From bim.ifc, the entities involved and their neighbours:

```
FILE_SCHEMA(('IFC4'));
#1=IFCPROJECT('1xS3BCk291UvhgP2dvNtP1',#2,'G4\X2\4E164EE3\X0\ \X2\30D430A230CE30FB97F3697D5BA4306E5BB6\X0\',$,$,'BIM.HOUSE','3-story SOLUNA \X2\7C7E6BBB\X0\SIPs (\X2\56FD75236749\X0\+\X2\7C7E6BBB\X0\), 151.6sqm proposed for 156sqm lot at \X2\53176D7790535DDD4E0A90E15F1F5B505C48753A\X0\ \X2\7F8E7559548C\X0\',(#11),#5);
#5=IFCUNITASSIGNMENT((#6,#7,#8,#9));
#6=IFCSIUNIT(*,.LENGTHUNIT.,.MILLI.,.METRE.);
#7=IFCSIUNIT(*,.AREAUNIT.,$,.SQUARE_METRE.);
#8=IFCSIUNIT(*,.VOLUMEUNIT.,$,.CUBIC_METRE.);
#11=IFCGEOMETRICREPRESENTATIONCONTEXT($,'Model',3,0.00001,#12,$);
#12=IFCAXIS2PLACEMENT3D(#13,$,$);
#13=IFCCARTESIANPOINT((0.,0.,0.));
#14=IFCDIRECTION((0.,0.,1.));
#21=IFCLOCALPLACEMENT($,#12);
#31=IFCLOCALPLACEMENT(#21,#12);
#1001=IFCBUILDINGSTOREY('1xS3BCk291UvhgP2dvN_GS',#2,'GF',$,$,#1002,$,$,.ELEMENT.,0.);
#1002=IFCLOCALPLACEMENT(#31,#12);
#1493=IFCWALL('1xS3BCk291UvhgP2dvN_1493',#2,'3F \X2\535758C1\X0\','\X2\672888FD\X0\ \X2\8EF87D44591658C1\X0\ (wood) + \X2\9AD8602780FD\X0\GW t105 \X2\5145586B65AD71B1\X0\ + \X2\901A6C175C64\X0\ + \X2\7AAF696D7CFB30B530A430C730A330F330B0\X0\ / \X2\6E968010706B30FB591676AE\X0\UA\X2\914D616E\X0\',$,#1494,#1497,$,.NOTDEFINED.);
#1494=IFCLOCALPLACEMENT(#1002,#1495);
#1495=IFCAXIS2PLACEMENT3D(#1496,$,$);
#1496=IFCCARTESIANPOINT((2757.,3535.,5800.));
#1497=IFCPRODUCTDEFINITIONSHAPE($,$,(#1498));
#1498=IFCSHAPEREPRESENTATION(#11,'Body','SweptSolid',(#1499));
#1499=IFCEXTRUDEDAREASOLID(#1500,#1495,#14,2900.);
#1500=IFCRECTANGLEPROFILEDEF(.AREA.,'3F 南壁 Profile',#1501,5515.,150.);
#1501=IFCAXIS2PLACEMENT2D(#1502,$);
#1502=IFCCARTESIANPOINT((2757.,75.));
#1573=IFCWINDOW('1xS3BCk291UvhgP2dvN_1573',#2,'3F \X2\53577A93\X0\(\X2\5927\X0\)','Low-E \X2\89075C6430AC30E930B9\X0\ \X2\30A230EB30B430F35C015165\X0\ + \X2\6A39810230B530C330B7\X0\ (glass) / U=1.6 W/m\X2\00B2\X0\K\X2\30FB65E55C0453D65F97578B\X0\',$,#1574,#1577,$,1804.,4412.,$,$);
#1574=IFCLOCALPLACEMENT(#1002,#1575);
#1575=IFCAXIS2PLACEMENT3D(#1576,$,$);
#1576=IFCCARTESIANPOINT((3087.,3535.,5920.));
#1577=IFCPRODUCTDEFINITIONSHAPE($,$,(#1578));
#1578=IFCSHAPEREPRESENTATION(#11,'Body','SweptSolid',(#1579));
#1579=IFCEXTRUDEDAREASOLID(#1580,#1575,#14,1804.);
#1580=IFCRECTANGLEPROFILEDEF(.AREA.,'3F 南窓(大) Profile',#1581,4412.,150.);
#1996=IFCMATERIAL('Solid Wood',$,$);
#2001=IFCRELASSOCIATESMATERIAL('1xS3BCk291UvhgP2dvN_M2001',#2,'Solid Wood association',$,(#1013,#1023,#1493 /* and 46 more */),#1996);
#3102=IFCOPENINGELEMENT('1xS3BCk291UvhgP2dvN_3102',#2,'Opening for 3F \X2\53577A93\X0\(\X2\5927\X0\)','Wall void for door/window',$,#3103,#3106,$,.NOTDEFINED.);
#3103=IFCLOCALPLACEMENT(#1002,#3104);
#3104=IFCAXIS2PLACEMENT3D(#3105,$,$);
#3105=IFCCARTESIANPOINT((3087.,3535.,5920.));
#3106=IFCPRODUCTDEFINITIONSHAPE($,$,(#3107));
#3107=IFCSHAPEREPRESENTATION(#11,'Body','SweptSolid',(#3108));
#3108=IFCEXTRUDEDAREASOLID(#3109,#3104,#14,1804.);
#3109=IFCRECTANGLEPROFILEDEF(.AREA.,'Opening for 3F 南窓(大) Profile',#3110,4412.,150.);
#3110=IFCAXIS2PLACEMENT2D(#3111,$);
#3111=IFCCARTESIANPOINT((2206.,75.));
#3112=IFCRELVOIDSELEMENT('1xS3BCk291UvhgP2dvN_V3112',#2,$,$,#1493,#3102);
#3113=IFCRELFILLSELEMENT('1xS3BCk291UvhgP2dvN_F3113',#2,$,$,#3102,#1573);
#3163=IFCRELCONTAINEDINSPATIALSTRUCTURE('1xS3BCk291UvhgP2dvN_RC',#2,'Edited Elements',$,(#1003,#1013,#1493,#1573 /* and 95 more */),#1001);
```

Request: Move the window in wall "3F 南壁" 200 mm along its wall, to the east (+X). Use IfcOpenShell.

```python
import ifcopenshell
import ifcopenshell.api.geometry
import ifcopenshell.util.placement
import ifcopenshell.util.unit

model = ifcopenshell.open("bim.ifc")
unit_scale = ifcopenshell.util.unit.calculate_unit_scale(model)

window = model.by_guid("1xS3BCk291UvhgP2dvN_1573")
opening = window.FillsVoids[0].RelatingOpeningElement
wall = opening.VoidsElements[0].RelatingBuildingElement

wall_matrix = ifcopenshell.util.placement.get_local_placement(wall.ObjectPlacement)
shift = wall_matrix[:3, 0] * 0.2 / unit_scale
before = ifcopenshell.util.placement.get_local_placement(window.ObjectPlacement)[:3, 3].copy()

# The window is not placed relative to its opening, so move both.
for product in (opening, window):
    matrix = ifcopenshell.util.placement.get_local_placement(product.ObjectPlacement)
    matrix[:3, 3] += shift
    ifcopenshell.api.geometry.edit_object_placement(model, product=product, matrix=matrix, is_si=False)

after = ifcopenshell.util.placement.get_local_placement(window.ObjectPlacement)[:3, 3]
print("window moved by", (after - before).round(3) + 0.0)

model.write("bim_rev.ifc")
```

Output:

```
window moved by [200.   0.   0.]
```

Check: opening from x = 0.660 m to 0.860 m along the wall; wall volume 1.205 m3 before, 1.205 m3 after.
